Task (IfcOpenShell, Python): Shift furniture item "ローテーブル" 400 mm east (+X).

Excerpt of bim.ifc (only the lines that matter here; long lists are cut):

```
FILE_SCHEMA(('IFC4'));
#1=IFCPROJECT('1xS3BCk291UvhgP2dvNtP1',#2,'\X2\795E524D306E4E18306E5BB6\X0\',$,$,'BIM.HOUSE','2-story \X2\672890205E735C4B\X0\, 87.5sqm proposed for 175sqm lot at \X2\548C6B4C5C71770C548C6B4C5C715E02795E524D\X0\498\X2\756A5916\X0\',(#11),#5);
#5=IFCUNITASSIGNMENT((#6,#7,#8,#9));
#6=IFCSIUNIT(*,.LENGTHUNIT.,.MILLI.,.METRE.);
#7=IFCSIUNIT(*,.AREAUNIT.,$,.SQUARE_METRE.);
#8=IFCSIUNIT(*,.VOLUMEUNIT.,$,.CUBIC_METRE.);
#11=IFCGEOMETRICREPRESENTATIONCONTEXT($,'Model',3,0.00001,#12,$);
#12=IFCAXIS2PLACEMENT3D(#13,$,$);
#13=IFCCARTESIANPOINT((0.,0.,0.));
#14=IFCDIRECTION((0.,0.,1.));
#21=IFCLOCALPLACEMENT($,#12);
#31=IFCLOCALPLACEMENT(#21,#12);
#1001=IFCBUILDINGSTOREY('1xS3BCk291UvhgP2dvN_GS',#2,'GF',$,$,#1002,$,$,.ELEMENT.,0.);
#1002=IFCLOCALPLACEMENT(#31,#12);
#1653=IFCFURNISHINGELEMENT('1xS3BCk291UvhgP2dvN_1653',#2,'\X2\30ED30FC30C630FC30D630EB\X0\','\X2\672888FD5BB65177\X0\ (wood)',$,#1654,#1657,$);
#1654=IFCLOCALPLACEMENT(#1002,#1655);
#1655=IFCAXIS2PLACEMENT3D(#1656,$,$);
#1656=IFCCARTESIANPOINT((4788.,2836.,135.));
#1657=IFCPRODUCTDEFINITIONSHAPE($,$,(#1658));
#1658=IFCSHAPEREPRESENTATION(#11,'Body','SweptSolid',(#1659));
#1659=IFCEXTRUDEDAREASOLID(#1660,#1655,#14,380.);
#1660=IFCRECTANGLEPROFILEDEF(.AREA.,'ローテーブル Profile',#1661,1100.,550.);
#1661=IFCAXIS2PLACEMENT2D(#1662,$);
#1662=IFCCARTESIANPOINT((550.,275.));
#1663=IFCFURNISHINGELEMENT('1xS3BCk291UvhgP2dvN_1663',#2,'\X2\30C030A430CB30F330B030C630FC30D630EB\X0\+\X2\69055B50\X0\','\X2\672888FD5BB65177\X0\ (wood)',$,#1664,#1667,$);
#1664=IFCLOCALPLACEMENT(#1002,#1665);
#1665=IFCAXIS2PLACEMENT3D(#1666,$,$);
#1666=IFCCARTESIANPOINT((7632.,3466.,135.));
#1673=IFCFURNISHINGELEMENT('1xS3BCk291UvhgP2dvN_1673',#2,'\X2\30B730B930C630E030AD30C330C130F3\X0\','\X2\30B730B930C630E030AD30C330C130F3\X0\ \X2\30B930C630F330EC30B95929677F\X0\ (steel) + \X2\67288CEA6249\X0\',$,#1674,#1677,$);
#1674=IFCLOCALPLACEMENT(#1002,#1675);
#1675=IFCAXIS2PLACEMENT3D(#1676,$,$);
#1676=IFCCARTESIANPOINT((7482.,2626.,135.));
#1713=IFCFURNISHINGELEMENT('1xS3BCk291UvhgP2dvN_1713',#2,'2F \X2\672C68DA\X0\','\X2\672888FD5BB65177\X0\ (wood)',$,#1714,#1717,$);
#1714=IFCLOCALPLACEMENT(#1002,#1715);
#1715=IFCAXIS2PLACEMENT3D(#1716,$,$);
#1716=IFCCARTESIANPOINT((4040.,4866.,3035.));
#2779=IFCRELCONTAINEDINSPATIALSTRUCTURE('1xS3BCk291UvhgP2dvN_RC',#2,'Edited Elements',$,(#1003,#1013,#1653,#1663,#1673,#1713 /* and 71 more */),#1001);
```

```python
import ifcopenshell
import ifcopenshell.api.geometry
import ifcopenshell.util.placement
import ifcopenshell.util.unit

model = ifcopenshell.open("bim.ifc")
unit_scale = ifcopenshell.util.unit.calculate_unit_scale(model)

item = model.by_guid("1xS3BCk291UvhgP2dvN_1653")
matrix = ifcopenshell.util.placement.get_local_placement(item.ObjectPlacement)
matrix[0, 3] += 0.4 / unit_scale
ifcopenshell.api.geometry.edit_object_placement(model, product=item, matrix=matrix, is_si=False)

print(ifcopenshell.util.placement.get_local_placement(item.ObjectPlacement).round(3) + 0.0)

model.write("bim_updated.ifc")
```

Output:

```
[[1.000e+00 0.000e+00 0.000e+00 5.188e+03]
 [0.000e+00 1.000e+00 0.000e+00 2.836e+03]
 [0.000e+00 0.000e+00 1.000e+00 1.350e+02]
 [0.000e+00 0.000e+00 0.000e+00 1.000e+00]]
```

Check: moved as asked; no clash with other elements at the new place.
